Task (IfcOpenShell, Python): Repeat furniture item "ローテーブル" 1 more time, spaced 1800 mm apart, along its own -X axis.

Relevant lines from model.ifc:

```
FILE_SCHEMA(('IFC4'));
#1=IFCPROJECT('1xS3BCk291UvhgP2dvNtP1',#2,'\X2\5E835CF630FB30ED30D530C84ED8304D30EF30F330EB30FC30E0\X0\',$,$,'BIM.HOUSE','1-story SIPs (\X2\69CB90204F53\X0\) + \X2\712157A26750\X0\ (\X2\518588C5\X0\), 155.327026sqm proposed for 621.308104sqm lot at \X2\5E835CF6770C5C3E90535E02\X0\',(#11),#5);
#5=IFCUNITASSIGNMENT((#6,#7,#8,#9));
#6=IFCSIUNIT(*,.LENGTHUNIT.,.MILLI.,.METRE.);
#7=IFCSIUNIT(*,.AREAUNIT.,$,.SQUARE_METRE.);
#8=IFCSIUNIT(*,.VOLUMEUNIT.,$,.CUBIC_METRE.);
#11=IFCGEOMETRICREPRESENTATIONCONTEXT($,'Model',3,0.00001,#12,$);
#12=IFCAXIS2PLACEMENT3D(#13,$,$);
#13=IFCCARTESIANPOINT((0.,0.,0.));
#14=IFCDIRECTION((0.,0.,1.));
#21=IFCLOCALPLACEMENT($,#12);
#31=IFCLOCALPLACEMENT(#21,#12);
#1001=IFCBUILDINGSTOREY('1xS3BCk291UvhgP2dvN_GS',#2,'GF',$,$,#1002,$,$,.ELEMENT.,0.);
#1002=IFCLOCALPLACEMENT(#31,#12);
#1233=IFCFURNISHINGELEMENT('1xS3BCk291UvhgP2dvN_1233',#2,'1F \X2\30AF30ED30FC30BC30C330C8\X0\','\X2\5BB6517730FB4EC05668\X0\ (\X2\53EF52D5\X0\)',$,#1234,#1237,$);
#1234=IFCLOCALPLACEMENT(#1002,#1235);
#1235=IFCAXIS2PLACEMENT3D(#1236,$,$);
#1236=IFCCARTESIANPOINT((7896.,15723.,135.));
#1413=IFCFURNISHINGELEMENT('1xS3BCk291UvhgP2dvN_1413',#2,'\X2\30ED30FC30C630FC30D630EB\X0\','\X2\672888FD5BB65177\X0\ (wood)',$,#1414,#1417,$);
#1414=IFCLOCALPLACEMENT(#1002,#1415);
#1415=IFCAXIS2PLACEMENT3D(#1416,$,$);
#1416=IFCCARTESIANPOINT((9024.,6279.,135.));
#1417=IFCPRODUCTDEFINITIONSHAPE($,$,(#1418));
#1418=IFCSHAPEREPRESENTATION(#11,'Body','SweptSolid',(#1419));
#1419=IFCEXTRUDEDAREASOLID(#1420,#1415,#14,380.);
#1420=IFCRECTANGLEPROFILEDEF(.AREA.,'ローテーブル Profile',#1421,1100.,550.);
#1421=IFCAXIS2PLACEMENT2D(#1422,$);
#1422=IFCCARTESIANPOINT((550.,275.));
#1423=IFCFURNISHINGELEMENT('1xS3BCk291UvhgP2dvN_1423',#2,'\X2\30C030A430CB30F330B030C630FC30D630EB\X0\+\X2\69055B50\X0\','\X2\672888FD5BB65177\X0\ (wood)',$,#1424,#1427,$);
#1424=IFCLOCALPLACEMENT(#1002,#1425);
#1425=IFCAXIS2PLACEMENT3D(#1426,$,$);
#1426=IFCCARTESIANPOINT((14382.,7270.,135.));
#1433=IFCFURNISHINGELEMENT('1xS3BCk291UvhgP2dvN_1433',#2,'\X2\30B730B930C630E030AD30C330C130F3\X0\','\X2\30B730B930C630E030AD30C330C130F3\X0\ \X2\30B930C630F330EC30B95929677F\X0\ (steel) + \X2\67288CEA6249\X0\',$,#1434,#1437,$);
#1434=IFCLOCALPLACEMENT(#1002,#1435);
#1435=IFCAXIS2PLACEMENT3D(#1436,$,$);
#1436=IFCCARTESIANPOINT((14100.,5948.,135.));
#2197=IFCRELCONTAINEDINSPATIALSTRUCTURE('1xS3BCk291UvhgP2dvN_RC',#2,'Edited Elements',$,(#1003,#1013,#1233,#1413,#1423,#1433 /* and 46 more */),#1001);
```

```python
import ifcopenshell
import ifcopenshell.api.geometry
import ifcopenshell.api.root
import ifcopenshell.util.element
import ifcopenshell.util.placement
import ifcopenshell.util.unit

model = ifcopenshell.open("model.ifc")
unit_scale = ifcopenshell.util.unit.calculate_unit_scale(model)


def reuse_history(source, copy):
    """copy_class also copies each property set's owner history, people and application; keep the originals."""
    for rel in copy.IsDefinedBy:
        if rel.is_a("IfcRelDefinesByProperties") and (history := rel.RelatingPropertyDefinition.OwnerHistory):
            rel.RelatingPropertyDefinition.OwnerHistory = source.OwnerHistory
            ifcopenshell.util.element.remove_deep2(model, history)


source = model.by_guid("1xS3BCk291UvhgP2dvN_1413")
base = ifcopenshell.util.placement.get_local_placement(source.ObjectPlacement)
step = -base[:3, 0] * 1.8 / unit_scale

for i in range(1, 2):
    copy = ifcopenshell.api.root.copy_class(model, product=source)
    copy.Representation = ifcopenshell.util.element.copy_deep(
        model, source.Representation, exclude=["IfcGeometricRepresentationContext", "IfcRepresentationMap"]
    )
    reuse_history(source, copy)
    matrix = base.copy()
    matrix[:3, 3] += i * step
    print("added at", matrix[:3, 3].round(3) + 0.0)
    ifcopenshell.api.geometry.edit_object_placement(model, product=copy, matrix=matrix, is_si=False)

model.write("model-out.ifc")
```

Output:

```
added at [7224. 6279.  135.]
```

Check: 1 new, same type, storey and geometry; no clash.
